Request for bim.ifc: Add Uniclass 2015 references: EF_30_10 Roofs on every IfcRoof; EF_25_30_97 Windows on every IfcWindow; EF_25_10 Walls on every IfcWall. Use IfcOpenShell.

First a look at what the model holds.

```python
import ifcopenshell

model = ifcopenshell.open("bim.ifc")
print(model.schema)
print("classifications:", [c.Name for c in model.by_type("IfcClassification")])
for ifc_class in ("IfcDoor", "IfcRoof", "IfcStair", "IfcWall", "IfcWindow"):
    print(ifc_class, len(model.by_type(ifc_class)))
```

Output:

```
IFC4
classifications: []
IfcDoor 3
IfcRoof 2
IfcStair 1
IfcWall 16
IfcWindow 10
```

```python
import ifcopenshell
import ifcopenshell.api.classification

model = ifcopenshell.open("bim.ifc")

system = ifcopenshell.api.classification.add_classification(model, classification="Uniclass 2015")

codes = {
    "IfcRoof": ("EF_30_10", "Roofs"),
    "IfcWindow": ("EF_25_30_97", "Windows"),
    "IfcWall": ("EF_25_10", "Walls"),
}
for ifc_class, (code, name) in codes.items():
    products = model.by_type(ifc_class)
    ifcopenshell.api.classification.add_reference(
        model, products=products, classification=system, identification=code, name=name
    )
    print(code, len(products))

model.write("bim_rev.ifc")
```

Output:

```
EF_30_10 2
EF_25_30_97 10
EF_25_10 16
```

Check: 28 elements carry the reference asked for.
